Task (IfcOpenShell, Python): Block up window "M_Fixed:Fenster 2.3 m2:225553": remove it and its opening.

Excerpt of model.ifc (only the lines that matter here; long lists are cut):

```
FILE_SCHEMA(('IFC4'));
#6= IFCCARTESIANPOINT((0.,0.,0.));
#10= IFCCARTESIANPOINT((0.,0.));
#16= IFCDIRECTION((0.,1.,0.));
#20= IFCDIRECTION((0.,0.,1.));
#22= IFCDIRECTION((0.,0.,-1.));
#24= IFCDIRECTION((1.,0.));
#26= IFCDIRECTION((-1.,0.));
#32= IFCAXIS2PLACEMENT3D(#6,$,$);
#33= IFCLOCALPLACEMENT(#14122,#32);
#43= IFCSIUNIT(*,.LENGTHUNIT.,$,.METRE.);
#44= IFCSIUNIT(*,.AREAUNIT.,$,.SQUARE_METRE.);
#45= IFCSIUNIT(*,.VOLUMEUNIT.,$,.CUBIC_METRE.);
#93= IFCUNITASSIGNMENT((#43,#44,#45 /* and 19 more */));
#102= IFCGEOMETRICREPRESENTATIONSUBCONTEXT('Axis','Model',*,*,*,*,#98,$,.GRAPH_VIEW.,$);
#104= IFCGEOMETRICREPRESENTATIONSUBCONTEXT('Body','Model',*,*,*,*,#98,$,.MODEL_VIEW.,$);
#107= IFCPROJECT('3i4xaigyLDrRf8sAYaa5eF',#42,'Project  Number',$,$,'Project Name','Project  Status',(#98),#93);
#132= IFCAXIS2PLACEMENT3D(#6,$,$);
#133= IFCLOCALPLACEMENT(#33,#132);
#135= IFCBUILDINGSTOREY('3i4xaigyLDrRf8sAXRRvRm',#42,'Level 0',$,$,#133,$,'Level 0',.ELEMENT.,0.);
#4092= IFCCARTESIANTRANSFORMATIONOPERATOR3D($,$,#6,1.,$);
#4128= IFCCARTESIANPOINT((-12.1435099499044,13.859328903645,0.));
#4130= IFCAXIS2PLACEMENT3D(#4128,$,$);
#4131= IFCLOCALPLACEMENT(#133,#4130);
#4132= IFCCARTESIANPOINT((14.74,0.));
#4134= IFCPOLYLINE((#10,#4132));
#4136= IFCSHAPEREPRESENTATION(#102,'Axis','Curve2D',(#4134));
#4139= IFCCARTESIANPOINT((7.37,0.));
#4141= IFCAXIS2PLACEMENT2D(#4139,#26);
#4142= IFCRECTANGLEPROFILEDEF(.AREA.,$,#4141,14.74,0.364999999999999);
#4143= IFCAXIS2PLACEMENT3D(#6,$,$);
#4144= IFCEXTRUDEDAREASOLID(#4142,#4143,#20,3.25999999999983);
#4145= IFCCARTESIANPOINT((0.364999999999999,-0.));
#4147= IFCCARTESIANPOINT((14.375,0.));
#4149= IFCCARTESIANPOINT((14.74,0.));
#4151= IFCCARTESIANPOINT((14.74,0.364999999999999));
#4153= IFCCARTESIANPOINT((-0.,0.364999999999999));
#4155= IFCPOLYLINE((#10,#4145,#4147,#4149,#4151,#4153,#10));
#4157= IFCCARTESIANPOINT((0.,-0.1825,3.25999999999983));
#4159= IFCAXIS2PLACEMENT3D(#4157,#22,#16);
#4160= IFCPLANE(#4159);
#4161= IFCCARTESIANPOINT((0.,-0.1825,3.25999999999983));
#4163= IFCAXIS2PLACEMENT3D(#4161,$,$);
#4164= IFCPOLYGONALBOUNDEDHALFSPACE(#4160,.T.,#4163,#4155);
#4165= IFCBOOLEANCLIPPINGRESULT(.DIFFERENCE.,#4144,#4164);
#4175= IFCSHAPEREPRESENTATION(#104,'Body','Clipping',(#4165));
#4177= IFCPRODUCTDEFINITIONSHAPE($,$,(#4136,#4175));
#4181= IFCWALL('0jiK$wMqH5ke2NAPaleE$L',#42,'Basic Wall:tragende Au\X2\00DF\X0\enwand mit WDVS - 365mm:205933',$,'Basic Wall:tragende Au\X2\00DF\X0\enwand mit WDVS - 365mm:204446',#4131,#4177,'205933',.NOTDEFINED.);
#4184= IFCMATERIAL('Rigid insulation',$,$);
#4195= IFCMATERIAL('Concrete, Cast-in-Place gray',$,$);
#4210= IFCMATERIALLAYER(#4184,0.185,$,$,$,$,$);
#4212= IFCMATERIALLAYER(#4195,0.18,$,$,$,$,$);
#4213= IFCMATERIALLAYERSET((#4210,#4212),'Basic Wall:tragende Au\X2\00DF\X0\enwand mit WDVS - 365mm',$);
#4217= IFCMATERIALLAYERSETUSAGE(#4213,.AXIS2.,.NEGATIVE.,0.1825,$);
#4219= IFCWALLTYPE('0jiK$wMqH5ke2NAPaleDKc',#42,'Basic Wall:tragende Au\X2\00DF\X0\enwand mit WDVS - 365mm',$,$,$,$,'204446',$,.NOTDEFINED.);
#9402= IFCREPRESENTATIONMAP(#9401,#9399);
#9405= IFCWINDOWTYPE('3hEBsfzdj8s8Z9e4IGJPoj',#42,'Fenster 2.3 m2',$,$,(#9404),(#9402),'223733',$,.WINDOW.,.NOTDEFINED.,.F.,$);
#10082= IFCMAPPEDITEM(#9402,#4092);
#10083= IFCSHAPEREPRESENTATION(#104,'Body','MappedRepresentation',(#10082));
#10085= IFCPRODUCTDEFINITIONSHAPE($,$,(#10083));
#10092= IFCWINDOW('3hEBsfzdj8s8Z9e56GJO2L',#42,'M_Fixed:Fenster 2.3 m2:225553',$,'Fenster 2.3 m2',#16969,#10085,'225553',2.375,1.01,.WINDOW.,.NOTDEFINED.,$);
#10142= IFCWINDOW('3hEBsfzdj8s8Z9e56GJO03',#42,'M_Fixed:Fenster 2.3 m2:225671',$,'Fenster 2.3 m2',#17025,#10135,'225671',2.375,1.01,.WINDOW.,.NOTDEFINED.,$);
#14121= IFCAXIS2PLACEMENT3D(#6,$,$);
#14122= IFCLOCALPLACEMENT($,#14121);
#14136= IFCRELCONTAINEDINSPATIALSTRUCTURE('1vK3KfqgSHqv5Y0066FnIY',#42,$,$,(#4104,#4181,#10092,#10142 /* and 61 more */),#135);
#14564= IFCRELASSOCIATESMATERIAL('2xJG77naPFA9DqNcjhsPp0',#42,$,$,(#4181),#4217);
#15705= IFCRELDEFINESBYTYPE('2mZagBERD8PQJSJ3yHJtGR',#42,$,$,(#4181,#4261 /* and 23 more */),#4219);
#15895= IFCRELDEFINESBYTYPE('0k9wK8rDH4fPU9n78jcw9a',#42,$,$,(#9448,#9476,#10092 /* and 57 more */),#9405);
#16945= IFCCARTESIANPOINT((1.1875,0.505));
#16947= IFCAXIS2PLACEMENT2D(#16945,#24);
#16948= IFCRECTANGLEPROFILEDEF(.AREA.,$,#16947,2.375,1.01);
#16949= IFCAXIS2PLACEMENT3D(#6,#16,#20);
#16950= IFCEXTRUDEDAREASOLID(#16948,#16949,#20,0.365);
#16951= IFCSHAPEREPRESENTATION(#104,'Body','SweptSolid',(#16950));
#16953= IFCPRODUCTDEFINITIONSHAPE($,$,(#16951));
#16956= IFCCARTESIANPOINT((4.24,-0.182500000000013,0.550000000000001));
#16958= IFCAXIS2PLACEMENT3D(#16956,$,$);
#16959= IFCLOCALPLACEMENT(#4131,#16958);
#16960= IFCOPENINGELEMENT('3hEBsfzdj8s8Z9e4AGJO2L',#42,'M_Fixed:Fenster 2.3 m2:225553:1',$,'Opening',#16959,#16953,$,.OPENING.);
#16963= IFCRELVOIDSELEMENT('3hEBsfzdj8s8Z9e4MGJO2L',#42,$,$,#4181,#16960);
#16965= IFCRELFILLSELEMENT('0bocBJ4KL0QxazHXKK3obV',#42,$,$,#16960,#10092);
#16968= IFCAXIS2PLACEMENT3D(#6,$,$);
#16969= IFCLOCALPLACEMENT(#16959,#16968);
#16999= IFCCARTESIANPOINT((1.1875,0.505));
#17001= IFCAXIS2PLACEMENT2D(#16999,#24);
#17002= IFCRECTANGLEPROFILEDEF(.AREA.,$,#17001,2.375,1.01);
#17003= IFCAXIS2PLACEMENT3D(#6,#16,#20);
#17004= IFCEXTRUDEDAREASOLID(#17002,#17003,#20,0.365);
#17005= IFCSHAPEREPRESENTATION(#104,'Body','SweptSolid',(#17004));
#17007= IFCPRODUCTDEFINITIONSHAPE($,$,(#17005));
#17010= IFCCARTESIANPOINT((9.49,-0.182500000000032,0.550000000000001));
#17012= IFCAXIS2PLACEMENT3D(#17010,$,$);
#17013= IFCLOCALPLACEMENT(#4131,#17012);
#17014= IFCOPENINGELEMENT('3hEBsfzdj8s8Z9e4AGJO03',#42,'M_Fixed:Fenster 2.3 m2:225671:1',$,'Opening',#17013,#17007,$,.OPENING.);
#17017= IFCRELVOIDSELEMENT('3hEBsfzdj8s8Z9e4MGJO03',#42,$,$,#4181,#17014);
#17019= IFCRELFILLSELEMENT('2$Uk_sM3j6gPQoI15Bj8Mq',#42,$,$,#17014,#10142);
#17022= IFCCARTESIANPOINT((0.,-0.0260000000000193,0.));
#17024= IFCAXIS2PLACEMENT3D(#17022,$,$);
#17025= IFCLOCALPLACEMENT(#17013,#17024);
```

```python
import ifcopenshell
import ifcopenshell.api.feature
import ifcopenshell.api.root
import ifcopenshell.geom
import ifcopenshell.util.shape

model = ifcopenshell.open("model.ifc")
settings = ifcopenshell.geom.settings()


def volume(element):
    """Net volume in cubic metres, openings subtracted."""
    shape = ifcopenshell.geom.create_shape(settings, element)
    return ifcopenshell.util.shape.get_volume(shape.geometry)


window = model.by_id(10092)
opening = window.FillsVoids[0].RelatingOpeningElement
wall = opening.VoidsElements[0].RelatingBuildingElement
before = volume(wall)

ifcopenshell.api.root.remove_product(model, product=window)
ifcopenshell.api.feature.remove_feature(model, feature=opening)

after = volume(wall)

print(f"wall volume {before:.3f} -> {after:.3f} m3")

model.write("model_edited.ifc")
```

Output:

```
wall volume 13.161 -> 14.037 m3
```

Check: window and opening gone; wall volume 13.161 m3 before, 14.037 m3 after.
